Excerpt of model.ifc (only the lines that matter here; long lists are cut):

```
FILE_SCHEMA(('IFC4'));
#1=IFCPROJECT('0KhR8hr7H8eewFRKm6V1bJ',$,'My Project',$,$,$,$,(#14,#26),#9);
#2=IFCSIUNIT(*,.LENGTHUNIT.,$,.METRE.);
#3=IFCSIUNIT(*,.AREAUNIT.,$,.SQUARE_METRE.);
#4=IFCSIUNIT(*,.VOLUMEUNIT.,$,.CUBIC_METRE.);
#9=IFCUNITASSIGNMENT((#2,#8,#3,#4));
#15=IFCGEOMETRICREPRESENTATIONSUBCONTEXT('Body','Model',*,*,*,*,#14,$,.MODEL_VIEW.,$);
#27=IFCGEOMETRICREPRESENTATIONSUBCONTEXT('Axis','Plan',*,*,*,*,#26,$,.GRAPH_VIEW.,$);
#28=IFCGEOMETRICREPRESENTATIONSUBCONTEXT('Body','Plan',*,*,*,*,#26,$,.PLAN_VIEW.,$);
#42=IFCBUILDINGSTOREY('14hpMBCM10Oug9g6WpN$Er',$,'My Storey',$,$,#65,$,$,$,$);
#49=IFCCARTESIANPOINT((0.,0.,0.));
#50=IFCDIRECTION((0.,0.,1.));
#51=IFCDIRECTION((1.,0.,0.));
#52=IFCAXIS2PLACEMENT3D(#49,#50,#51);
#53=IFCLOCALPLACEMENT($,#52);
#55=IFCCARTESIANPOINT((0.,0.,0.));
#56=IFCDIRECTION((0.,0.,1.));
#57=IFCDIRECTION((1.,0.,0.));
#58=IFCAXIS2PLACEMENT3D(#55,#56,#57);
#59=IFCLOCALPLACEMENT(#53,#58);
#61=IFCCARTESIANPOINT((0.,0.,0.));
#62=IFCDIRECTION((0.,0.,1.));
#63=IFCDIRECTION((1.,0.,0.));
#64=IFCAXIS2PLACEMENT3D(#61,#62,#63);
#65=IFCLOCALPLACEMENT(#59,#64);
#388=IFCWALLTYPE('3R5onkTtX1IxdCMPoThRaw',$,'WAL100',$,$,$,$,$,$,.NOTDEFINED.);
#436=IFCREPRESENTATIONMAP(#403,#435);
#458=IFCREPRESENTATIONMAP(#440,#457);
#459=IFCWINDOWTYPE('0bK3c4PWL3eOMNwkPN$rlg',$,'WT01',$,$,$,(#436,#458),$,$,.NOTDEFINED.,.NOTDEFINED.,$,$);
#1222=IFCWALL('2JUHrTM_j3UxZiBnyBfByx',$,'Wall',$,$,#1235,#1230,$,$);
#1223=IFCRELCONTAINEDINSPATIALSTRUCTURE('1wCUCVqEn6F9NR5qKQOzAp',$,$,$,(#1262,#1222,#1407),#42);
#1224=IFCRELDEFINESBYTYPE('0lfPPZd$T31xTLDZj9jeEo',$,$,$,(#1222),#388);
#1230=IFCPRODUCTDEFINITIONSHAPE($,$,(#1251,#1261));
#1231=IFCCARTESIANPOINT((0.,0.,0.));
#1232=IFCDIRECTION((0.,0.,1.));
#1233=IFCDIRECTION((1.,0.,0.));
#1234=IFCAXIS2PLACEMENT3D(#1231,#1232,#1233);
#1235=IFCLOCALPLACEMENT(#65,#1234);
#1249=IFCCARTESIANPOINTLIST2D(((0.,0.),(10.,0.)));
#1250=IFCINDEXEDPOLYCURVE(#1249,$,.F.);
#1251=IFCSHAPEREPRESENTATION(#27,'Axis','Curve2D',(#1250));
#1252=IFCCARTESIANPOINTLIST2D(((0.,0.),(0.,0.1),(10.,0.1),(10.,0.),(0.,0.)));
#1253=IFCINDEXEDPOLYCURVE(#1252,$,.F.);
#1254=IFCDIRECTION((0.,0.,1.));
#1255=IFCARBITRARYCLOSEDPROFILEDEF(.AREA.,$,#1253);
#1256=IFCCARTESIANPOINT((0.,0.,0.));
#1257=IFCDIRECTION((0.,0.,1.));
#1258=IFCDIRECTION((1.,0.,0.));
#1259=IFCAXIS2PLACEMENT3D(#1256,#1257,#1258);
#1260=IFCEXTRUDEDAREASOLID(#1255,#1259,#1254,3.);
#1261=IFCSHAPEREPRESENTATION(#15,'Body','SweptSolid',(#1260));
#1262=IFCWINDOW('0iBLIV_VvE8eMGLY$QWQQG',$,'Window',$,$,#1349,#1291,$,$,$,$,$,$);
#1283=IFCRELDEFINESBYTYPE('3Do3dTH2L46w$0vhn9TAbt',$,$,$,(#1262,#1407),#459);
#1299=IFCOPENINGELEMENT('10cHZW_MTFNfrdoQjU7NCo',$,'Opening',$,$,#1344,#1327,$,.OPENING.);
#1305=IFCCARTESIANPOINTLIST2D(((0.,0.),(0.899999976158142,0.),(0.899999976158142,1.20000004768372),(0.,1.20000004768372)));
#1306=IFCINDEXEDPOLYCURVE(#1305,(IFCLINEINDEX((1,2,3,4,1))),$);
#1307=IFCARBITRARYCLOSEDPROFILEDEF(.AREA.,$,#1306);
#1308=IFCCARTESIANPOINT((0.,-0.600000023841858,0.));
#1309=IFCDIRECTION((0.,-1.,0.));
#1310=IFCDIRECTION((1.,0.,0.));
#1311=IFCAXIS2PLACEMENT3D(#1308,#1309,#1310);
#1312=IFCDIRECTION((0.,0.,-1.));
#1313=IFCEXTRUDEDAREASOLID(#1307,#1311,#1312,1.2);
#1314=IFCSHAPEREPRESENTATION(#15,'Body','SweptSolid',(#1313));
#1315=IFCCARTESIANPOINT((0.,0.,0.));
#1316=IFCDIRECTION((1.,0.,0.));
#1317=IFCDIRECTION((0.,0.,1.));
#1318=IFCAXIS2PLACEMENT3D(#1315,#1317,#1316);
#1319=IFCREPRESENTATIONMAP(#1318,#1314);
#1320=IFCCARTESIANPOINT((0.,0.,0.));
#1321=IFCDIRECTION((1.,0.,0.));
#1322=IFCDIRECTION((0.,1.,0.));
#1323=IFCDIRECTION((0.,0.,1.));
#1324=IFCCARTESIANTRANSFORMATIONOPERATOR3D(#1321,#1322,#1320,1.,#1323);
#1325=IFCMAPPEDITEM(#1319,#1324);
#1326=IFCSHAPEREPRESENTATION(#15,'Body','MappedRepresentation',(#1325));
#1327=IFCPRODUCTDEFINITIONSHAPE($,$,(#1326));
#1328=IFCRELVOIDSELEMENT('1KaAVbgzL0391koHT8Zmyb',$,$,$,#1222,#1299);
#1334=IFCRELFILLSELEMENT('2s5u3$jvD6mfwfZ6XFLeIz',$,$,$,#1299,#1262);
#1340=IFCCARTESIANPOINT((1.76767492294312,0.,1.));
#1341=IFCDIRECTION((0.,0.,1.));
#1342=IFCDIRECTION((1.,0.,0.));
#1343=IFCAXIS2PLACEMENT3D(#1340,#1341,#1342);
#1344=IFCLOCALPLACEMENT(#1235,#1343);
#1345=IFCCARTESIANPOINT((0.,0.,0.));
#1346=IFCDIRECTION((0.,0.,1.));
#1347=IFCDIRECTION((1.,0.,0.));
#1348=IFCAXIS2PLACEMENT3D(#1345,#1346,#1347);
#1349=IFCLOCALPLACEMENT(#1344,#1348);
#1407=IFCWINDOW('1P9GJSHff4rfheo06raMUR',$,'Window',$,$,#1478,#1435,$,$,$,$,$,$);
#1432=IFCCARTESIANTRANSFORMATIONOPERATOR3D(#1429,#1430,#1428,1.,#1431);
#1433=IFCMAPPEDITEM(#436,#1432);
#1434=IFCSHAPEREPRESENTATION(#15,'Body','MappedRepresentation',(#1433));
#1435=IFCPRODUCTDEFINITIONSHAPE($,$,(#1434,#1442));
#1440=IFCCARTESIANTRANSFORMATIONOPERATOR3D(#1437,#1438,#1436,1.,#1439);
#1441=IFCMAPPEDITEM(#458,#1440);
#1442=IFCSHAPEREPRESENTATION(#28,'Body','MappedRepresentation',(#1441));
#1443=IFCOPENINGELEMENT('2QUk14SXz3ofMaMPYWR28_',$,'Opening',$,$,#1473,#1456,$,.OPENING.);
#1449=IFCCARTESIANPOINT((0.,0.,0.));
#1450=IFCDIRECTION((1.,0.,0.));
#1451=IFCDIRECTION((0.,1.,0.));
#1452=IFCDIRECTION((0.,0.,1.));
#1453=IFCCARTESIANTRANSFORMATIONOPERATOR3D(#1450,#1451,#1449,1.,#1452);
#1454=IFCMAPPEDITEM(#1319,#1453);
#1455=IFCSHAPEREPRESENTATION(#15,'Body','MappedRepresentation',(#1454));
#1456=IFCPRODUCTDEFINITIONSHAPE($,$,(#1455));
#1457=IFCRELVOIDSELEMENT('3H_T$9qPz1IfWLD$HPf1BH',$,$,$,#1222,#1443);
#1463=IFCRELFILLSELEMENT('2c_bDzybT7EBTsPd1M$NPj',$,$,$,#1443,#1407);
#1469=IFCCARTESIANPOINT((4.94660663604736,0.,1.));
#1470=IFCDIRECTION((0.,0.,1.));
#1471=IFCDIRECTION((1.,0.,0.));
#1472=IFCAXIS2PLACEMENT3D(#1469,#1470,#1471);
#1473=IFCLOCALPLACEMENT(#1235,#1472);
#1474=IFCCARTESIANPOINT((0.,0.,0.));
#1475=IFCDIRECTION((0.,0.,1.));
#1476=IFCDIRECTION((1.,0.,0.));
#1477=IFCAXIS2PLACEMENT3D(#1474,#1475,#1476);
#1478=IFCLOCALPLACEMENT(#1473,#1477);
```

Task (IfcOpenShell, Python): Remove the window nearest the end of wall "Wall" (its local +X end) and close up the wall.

```python
import ifcopenshell
import ifcopenshell.api.feature
import ifcopenshell.api.root
import ifcopenshell.geom
import ifcopenshell.util.shape

model = ifcopenshell.open("model.ifc")
settings = ifcopenshell.geom.settings()


def volume(element):
    """Net volume in cubic metres, openings subtracted."""
    shape = ifcopenshell.geom.create_shape(settings, element)
    return ifcopenshell.util.shape.get_volume(shape.geometry)


window = model.by_id(1407)
opening = window.FillsVoids[0].RelatingOpeningElement
wall = opening.VoidsElements[0].RelatingBuildingElement
before = volume(wall)

ifcopenshell.api.root.remove_product(model, product=window)
ifcopenshell.api.feature.remove_feature(model, feature=opening)

after = volume(wall)

print(f"wall volume {before:.3f} -> {after:.3f} m3")

model.write("model_updated.ifc")
```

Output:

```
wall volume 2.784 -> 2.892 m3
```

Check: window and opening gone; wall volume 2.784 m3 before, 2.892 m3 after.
